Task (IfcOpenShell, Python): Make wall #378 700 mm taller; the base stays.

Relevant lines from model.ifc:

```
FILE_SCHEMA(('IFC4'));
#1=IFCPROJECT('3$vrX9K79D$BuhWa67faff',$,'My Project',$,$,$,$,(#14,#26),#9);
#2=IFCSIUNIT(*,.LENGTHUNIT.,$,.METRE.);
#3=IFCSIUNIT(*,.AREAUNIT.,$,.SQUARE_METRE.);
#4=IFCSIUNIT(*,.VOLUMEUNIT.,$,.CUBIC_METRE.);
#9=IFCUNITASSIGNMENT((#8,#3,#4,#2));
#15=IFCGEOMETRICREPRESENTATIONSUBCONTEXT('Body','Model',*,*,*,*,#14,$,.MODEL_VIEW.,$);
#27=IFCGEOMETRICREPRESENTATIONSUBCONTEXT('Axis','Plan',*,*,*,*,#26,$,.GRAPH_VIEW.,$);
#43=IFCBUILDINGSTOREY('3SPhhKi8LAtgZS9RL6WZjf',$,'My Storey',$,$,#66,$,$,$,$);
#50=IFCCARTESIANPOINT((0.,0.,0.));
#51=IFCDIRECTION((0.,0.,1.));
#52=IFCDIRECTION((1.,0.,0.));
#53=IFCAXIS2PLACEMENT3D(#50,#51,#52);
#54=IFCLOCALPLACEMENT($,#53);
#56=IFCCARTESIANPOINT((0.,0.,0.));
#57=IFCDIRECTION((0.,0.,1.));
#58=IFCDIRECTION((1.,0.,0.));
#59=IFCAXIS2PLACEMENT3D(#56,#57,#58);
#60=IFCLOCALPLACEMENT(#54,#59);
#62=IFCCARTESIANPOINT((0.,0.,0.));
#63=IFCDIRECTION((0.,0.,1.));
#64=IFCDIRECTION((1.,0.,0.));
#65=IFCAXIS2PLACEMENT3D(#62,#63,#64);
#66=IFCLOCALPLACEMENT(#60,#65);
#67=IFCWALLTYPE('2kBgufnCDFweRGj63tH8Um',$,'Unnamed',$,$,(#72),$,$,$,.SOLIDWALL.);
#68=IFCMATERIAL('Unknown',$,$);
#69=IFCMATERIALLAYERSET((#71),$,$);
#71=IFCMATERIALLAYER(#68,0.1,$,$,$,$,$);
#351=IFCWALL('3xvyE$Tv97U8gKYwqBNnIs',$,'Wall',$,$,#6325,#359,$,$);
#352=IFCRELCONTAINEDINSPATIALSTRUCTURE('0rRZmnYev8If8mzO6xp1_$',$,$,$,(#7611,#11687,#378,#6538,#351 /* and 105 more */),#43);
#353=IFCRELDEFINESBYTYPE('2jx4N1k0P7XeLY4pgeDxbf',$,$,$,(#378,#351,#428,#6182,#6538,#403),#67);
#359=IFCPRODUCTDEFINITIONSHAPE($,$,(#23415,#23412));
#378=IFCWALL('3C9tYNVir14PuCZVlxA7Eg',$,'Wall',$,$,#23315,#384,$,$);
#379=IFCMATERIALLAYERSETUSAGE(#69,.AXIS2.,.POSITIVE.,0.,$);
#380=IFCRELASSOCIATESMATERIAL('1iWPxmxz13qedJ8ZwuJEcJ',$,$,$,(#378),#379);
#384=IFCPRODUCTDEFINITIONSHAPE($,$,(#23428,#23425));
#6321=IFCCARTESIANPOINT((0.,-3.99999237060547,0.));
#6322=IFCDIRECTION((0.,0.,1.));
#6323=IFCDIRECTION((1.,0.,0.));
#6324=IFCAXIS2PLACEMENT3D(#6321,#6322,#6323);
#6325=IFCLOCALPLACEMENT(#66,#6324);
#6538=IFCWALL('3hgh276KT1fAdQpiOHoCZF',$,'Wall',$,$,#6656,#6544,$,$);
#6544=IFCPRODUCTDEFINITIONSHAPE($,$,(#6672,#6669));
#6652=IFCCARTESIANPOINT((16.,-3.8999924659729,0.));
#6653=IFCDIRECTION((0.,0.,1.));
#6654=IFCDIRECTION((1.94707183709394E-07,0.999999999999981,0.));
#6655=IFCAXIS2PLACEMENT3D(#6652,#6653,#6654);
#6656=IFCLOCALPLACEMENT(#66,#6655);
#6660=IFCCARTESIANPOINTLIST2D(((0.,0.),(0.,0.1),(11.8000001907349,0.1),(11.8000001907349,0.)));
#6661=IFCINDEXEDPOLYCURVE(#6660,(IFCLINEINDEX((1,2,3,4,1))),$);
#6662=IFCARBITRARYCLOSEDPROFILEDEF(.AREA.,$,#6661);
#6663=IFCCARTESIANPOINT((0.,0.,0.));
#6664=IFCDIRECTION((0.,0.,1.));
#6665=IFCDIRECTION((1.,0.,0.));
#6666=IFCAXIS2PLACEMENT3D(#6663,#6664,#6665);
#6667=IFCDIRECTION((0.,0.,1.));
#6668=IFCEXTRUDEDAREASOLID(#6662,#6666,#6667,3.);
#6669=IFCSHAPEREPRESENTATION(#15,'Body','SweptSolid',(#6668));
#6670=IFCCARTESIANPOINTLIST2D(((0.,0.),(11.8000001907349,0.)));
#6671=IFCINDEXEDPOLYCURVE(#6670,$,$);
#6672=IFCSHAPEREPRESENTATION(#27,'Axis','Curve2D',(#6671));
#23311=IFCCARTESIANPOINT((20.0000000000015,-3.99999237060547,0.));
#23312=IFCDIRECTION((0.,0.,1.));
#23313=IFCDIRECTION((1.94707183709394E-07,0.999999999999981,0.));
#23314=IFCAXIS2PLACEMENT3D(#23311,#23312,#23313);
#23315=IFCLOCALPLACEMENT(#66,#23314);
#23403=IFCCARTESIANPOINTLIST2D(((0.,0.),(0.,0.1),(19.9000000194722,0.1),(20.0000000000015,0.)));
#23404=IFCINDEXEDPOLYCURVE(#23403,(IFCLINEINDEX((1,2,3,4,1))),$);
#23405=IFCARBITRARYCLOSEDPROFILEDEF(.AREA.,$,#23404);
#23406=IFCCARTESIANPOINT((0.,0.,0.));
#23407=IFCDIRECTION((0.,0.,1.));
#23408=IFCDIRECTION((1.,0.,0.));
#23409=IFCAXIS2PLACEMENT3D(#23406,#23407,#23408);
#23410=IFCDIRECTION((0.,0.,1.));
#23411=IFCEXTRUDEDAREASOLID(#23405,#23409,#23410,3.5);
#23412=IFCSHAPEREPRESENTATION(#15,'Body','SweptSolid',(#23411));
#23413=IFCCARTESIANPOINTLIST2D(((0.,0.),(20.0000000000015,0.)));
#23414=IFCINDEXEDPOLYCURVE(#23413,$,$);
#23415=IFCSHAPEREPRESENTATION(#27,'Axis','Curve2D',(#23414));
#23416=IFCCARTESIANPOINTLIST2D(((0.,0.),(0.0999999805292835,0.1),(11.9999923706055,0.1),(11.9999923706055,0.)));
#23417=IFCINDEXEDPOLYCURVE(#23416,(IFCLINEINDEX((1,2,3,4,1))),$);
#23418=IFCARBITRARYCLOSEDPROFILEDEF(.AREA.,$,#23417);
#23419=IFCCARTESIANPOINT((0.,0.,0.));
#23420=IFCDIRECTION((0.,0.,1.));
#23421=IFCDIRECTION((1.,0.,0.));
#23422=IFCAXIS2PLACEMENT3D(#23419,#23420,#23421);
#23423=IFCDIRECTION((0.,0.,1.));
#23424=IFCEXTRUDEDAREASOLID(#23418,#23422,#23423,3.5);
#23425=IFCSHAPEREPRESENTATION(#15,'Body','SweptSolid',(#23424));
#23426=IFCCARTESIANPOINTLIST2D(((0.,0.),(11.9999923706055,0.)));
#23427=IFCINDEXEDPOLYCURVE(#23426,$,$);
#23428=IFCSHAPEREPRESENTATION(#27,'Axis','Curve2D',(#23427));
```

```python
import ifcopenshell
import ifcopenshell.geom
import ifcopenshell.util.representation
import ifcopenshell.util.shape
import ifcopenshell.util.unit

model = ifcopenshell.open("model.ifc")
unit_scale = ifcopenshell.util.unit.calculate_unit_scale(model)
settings = ifcopenshell.geom.settings()


def volume(element):
    """Net volume in cubic metres, openings subtracted."""
    shape = ifcopenshell.geom.create_shape(settings, element)
    return ifcopenshell.util.shape.get_volume(shape.geometry)


wall = model.by_id(378)
before = volume(wall)

body = ifcopenshell.util.representation.get_representation(wall, "Model", "Body")
solid = body.Items[0]
old_height = solid.Depth
solid.Depth += 0.7 / unit_scale
after = volume(wall)

print(f"height {old_height:g} -> {solid.Depth:g}, volume {before:.3f} -> {after:.3f} m3")

model.write("model-out.ifc")
```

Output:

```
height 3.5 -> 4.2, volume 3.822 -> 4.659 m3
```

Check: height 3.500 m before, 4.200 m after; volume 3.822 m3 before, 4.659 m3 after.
